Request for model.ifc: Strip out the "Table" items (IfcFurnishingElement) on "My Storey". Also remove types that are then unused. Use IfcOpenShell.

First a look at what the model holds.

```python
import ifcopenshell
import ifcopenshell.util.element

model = ifcopenshell.open("model.ifc")
print(model.schema)
storey = next(s for s in model.by_type("IfcBuildingStorey") if s.Name == "My Storey")
furniture = [e for e in ifcopenshell.util.element.get_decomposition(storey) if e.is_a("IfcFurnishingElement")]
seen = {}
for e in furniture:
    element_type = ifcopenshell.util.element.get_type(e)
    name = element_type.Name if element_type not in (None, e) else None
    seen[name] = seen.get(name, 0) + 1
for name, count in sorted(seen.items(), key=str):
    print(count, "x", name)
```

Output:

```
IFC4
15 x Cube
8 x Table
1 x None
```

```python
import ifcopenshell
import ifcopenshell.api.root
import ifcopenshell.util.element

model = ifcopenshell.open("model.ifc")

storey = next(s for s in model.by_type("IfcBuildingStorey") if s.Name == "My Storey")
furniture = [e for e in ifcopenshell.util.element.get_decomposition(storey) if e.is_a("IfcFurnishingElement")]
targets = [e for e in furniture if (t := ifcopenshell.util.element.get_type(e)) not in (None, e) and t.Name == "Table"]
types = {ifcopenshell.util.element.get_type(e) for e in targets} - {None, *targets}

for e in targets:
    ifcopenshell.api.root.remove_product(model, product=e)
print(len(targets), "removed")

unused = [t for t in types if not ifcopenshell.util.element.get_types(t)]
for t in unused:
    ifcopenshell.api.root.remove_product(model, product=t)
print(len(unused), "unused types removed")

model.write("model_rev.ifc")
```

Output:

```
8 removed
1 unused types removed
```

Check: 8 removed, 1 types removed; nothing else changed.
